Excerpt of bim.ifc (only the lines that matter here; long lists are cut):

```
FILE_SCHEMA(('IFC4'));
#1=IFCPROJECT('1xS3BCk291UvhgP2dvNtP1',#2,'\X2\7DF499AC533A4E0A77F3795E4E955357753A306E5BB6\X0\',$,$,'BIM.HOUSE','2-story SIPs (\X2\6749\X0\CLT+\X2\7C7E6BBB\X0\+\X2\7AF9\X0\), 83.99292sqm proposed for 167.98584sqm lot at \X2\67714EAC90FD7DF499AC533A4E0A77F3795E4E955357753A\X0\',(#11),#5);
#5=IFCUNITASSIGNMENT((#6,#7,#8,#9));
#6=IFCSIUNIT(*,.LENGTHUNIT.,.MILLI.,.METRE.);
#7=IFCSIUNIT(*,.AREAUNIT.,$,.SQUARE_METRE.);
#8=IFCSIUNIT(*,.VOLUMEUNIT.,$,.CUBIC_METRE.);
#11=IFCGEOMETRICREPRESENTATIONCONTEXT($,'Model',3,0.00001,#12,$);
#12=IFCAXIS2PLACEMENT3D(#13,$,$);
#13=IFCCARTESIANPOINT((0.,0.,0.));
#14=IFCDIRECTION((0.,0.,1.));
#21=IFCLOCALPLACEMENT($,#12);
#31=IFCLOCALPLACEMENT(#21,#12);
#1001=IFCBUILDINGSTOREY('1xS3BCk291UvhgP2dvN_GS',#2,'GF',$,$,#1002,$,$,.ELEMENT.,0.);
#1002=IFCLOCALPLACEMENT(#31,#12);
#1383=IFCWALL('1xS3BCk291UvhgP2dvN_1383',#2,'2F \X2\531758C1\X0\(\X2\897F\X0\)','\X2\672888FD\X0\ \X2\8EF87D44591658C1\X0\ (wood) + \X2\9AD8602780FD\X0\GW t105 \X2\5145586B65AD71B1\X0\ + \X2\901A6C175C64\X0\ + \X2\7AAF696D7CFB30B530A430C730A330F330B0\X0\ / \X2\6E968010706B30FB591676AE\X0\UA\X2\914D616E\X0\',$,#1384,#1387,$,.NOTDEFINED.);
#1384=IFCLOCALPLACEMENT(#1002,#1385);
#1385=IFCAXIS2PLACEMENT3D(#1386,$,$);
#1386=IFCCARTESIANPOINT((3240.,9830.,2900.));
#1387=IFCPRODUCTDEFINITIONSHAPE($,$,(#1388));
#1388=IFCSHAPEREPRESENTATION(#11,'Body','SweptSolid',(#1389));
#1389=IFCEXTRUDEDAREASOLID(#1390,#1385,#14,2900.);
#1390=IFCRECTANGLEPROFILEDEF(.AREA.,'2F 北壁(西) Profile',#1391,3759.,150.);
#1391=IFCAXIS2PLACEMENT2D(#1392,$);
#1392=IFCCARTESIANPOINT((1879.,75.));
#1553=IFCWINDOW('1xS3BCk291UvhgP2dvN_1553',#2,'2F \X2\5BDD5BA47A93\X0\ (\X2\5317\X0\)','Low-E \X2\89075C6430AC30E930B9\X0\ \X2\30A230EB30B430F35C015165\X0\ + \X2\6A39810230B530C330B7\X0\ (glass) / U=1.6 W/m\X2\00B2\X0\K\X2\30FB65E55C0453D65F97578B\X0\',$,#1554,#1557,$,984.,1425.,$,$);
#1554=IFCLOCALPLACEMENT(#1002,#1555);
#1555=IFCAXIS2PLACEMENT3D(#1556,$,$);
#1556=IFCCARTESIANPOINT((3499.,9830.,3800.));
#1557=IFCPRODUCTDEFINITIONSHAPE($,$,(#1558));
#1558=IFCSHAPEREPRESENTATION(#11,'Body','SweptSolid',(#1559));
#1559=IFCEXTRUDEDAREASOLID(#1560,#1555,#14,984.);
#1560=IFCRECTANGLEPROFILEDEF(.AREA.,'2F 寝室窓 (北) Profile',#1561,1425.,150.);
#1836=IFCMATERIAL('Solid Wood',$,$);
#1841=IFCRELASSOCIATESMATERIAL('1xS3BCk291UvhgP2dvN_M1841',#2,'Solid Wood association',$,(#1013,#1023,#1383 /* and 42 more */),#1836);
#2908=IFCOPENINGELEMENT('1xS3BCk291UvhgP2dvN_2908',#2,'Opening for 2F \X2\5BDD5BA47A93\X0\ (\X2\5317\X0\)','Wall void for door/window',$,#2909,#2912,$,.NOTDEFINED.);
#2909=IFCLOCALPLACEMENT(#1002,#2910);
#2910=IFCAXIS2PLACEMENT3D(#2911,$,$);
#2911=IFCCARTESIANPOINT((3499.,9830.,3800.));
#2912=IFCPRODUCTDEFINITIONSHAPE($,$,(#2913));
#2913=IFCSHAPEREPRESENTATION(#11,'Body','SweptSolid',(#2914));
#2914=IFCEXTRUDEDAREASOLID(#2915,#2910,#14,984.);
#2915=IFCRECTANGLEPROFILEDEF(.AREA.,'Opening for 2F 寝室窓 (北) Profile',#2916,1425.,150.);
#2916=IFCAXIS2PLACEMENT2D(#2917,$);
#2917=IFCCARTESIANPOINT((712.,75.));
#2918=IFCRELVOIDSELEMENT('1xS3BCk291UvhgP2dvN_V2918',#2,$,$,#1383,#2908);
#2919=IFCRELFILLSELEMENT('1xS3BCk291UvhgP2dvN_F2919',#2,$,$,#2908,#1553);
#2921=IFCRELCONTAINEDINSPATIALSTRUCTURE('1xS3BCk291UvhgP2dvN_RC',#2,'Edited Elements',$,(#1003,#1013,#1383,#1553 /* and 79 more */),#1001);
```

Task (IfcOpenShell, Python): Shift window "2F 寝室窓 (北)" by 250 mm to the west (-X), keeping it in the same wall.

```python
import ifcopenshell
import ifcopenshell.api.geometry
import ifcopenshell.util.placement

model = ifcopenshell.open("bim.ifc")

window = model.by_guid("1xS3BCk291UvhgP2dvN_1553")
opening = window.FillsVoids[0].RelatingOpeningElement
wall = opening.VoidsElements[0].RelatingBuildingElement

wall_matrix = ifcopenshell.util.placement.get_local_placement(wall.ObjectPlacement)
shift = wall_matrix[:3, 0] * -250.0
before = ifcopenshell.util.placement.get_local_placement(window.ObjectPlacement)[:3, 3].copy()

# The window is not placed relative to its opening, so move both.
for product in (opening, window):
    matrix = ifcopenshell.util.placement.get_local_placement(product.ObjectPlacement)
    matrix[:3, 3] += shift
    ifcopenshell.api.geometry.edit_object_placement(model, product=product, matrix=matrix, is_si=False)

after = ifcopenshell.util.placement.get_local_placement(window.ObjectPlacement)[:3, 3]
print("window moved by", (after - before).round(3) + 0.0)

model.write("bim_updated.ifc")
```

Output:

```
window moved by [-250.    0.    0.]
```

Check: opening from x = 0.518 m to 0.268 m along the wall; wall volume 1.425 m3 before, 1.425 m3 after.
